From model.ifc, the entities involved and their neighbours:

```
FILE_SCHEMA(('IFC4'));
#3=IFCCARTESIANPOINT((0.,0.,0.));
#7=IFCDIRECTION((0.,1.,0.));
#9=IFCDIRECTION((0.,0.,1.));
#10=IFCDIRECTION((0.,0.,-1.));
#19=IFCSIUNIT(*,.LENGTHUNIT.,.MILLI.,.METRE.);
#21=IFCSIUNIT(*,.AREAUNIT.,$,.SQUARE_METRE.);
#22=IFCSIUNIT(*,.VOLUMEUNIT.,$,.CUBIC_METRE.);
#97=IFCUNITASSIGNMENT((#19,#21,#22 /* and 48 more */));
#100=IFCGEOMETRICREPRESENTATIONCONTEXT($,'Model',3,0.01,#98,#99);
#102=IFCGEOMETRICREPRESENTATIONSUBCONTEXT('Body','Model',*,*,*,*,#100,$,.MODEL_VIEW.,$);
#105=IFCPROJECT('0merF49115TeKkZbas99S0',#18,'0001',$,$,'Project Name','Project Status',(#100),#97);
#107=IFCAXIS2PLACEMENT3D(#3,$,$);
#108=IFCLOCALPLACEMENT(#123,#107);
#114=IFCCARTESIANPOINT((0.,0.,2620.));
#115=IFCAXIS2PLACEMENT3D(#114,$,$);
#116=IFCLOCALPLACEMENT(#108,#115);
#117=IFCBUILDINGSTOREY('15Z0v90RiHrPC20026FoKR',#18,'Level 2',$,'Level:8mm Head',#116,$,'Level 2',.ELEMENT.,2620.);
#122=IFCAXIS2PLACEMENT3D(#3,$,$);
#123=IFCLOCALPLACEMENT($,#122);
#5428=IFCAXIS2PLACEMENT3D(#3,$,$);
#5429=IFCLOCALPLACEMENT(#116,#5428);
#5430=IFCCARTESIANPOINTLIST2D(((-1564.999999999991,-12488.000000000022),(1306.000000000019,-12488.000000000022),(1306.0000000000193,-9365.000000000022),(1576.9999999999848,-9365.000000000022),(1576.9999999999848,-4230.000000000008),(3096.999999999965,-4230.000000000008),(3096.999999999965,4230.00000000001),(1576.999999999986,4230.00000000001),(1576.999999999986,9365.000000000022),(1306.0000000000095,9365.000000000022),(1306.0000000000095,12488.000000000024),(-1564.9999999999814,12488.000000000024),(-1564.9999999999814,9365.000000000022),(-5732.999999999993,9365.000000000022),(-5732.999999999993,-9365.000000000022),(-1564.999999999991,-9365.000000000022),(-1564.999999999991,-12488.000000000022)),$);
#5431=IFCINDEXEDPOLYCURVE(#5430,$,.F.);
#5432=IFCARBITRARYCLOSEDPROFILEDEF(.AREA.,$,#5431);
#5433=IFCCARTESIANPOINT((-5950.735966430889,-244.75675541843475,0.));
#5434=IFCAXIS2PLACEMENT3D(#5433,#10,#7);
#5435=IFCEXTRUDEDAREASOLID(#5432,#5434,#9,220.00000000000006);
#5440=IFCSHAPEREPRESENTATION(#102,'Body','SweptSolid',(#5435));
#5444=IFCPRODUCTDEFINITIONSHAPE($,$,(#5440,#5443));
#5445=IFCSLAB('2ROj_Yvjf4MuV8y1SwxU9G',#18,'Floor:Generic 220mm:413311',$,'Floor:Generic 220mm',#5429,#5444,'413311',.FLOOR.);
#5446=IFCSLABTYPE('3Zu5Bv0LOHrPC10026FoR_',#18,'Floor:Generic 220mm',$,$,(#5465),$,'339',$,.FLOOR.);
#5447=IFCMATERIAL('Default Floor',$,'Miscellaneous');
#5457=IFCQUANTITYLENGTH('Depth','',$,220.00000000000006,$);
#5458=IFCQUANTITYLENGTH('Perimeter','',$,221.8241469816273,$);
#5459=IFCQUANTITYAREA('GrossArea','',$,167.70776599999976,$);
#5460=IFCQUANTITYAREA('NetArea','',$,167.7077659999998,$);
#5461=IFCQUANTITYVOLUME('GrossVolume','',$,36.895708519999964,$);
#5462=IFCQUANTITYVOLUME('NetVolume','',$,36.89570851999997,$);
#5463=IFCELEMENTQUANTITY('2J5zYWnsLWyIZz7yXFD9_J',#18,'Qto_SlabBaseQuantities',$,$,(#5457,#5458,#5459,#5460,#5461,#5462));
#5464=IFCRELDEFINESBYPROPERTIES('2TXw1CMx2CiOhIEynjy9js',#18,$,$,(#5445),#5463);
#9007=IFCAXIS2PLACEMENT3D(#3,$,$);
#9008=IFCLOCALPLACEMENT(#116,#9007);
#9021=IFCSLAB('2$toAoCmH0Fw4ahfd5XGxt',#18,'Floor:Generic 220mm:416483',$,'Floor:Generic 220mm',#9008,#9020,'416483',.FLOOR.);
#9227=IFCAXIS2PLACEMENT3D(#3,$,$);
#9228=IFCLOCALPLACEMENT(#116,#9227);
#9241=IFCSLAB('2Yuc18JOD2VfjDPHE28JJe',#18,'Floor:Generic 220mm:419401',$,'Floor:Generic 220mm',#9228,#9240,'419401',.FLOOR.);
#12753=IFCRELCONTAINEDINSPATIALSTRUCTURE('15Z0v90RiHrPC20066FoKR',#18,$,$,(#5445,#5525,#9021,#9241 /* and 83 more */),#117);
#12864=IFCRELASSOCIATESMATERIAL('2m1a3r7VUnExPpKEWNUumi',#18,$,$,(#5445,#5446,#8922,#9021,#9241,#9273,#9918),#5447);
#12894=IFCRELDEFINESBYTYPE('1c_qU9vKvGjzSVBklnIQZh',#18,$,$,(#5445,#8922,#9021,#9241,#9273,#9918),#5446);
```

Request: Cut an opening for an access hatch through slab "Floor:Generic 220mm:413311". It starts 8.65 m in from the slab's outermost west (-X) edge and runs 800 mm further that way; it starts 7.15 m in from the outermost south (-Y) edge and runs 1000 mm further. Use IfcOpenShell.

```python
import numpy as np
import ifcopenshell
import ifcopenshell.api.feature
import ifcopenshell.api.geometry
import ifcopenshell.api.pset
import ifcopenshell.api.root
import ifcopenshell.geom
import ifcopenshell.util.element
import ifcopenshell.util.placement
import ifcopenshell.util.representation
import ifcopenshell.util.shape
import ifcopenshell.util.unit

model = ifcopenshell.open("model.ifc")
unit_scale = ifcopenshell.util.unit.calculate_unit_scale(model)
area_scale = ifcopenshell.util.unit.calculate_unit_scale(model, "AREAUNIT")
volume_scale = ifcopenshell.util.unit.calculate_unit_scale(model, "VOLUMEUNIT")
settings = ifcopenshell.geom.settings()


def volume(element):
    """Net volume in cubic metres, openings subtracted."""
    shape = ifcopenshell.geom.create_shape(settings, element)
    return ifcopenshell.util.shape.get_volume(shape.geometry)


slab = model.by_guid("2ROj_Yvjf4MuV8y1SwxU9G")
before = volume(slab)

# Extent in the slab's own axes, in metres. The edges named are its -X and -Y sides.
slab_shape = ifcopenshell.geom.create_shape(settings, slab)
vertices = ifcopenshell.util.shape.get_vertices(slab_shape.geometry)
x_min, y_min, bottom = vertices.min(axis=0)
top = vertices[:, 2].max()

opening = ifcopenshell.api.root.create_entity(model, ifc_class="IfcOpeningElement", name="Access hatch opening", predefined_type="OPENING")
context = ifcopenshell.util.representation.get_context(model, "Model", "Body", "MODEL_VIEW")
width, depth = 0.8, 1
outline = [(0.0, 0.0), (width, 0.0), (width, depth), (0.0, depth), (0.0, 0.0)]
# Overshoot both faces by 50 mm so the cut is clean.
shape = ifcopenshell.api.geometry.add_slab_representation(
    model, context=context, depth=top - bottom + 0.1, polyline=outline
)
ifcopenshell.api.geometry.assign_representation(model, product=opening, representation=shape)

matrix = ifcopenshell.util.placement.get_local_placement(slab.ObjectPlacement)
matrix[:, 3] = matrix @ np.append(np.array([x_min + 8.65, y_min + 7.15, bottom - 0.05]) / unit_scale, 1.0)
ifcopenshell.api.geometry.edit_object_placement(model, product=opening, matrix=matrix, is_si=False)
ifcopenshell.api.feature.add_feature(model, feature=opening, element=slab)

after = volume(slab)

# Update the slab's stored quantities.
qto = model.by_id(ifcopenshell.util.element.get_pset(slab, "Qto_SlabBaseQuantities", should_inherit=False)["id"])
ifcopenshell.api.pset.edit_qto(model, qto=qto, properties={
    "NetArea": after / (top - bottom) / area_scale,
    "NetVolume": after / volume_scale,
})

print(f"slab volume {before:.3f} -> {after:.3f} m3")

model.write("model-out.ifc")
```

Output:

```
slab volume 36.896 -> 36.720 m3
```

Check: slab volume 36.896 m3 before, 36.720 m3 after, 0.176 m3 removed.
